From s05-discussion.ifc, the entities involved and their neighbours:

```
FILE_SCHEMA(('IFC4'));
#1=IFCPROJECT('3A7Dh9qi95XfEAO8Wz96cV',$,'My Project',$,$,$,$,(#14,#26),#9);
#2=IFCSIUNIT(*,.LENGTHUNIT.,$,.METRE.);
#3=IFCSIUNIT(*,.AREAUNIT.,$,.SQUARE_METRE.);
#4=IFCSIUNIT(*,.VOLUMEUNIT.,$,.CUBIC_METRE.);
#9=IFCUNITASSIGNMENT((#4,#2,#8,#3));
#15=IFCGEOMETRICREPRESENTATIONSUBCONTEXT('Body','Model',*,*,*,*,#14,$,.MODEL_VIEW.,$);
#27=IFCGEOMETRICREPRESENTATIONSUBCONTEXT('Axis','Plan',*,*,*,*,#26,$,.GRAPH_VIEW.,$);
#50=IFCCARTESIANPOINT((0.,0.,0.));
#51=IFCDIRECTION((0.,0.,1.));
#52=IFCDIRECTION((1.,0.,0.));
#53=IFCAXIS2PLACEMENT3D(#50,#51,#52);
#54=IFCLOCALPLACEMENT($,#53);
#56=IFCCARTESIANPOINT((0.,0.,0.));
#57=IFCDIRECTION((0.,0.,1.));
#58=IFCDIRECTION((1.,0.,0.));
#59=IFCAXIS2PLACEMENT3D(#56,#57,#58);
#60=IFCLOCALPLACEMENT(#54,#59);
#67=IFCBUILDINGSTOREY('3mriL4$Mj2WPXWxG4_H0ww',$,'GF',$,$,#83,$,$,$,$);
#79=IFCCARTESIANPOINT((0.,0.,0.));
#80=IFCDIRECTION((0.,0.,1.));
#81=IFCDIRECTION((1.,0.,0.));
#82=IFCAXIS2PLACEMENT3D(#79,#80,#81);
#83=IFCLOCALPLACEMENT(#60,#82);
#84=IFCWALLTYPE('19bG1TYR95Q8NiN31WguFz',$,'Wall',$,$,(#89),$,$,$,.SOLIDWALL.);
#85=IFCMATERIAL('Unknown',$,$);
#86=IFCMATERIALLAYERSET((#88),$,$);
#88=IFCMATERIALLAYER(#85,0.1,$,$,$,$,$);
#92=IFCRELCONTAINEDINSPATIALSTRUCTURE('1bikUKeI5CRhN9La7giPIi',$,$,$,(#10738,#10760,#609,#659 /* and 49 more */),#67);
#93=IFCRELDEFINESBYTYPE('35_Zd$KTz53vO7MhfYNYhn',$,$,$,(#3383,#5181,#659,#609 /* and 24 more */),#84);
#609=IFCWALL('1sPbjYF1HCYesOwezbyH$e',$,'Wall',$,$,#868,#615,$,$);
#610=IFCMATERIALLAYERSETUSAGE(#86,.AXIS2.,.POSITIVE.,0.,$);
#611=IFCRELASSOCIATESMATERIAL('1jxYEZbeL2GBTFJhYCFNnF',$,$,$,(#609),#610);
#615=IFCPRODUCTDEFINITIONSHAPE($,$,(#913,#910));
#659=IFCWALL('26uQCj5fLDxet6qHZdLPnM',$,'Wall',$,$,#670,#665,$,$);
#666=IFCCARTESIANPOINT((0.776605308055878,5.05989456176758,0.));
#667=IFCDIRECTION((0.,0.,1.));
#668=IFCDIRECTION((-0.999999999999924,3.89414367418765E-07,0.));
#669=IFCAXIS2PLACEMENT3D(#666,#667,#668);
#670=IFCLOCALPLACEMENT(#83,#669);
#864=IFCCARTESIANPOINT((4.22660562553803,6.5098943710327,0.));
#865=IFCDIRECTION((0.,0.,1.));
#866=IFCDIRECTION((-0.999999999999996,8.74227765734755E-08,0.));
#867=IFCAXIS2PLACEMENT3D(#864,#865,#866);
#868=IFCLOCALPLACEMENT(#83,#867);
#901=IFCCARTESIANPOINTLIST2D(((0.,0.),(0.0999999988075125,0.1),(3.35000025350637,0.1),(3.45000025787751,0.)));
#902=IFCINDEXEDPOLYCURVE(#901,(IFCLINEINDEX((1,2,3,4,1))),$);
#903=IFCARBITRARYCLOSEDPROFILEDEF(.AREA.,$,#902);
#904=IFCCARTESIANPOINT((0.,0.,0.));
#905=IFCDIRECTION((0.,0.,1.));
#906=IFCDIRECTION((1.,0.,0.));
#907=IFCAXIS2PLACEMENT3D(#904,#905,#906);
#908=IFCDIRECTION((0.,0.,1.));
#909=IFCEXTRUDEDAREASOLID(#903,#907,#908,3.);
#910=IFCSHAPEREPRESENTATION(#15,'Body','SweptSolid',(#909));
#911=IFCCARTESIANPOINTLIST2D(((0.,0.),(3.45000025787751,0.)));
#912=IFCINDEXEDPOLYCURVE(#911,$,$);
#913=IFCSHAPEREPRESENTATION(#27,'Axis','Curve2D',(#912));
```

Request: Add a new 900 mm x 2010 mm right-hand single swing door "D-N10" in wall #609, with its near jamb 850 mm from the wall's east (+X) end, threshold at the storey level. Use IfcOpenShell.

```python
import numpy as np
import ifcopenshell
import ifcopenshell.api.feature
import ifcopenshell.api.geometry
import ifcopenshell.api.root
import ifcopenshell.api.spatial
import ifcopenshell.geom
import ifcopenshell.util.element
import ifcopenshell.util.placement
import ifcopenshell.util.representation
import ifcopenshell.util.shape
import ifcopenshell.util.unit

model = ifcopenshell.open("s05-discussion.ifc")
unit_scale = ifcopenshell.util.unit.calculate_unit_scale(model)
settings = ifcopenshell.geom.settings()


def volume(element):
    """Net volume in cubic metres, openings subtracted."""
    shape = ifcopenshell.geom.create_shape(settings, element)
    return ifcopenshell.util.shape.get_volume(shape.geometry)


wall = model.by_id(609)
storey = ifcopenshell.util.element.get_container(wall, ifc_class="IfcBuildingStorey")
context = ifcopenshell.util.representation.get_context(model, "Model", "Body", "MODEL_VIEW")
before = volume(wall)

width, height, from_end, sill = 0.9, 2.01, 0.85, 0.0  # metres

# The wall runs along its own X axis, and the end named is its -X end.
wall_shape = ifcopenshell.geom.create_shape(settings, wall)
x, y, z = ifcopenshell.util.shape.get_vertices(wall_shape.geometry).T
start = x.min() + from_end
face, thickness = float(y.min()), float(y.max() - y.min())
wall_matrix = ifcopenshell.util.placement.get_local_placement(wall.ObjectPlacement)
level = ifcopenshell.util.placement.get_local_placement(storey.ObjectPlacement)[2, 3]


def in_wall(x, y):
    """Placement at x, y metres in the wall's axes, at sill height."""
    matrix = wall_matrix.copy()
    matrix[:, 3] = wall_matrix @ np.array([x / unit_scale, y / unit_scale, 0.0, 1.0])
    matrix[2, 3] = level + sill / unit_scale
    return matrix


# Opening: a box that overshoots both wall faces by 50 mm.
opening = ifcopenshell.api.root.create_entity(model, ifc_class="IfcOpeningElement", predefined_type="OPENING")
box = ifcopenshell.api.geometry.add_wall_representation(
    model, context=context, length=width, height=height, thickness=thickness + 0.1
)
ifcopenshell.api.geometry.assign_representation(model, product=opening, representation=box)
ifcopenshell.api.geometry.edit_object_placement(model, product=opening, matrix=in_wall(start, face - 0.05), is_si=False)
ifcopenshell.api.feature.add_feature(model, feature=opening, element=wall)

door = ifcopenshell.api.root.create_entity(model, ifc_class="IfcDoor", name="D-N10", predefined_type="DOOR")
door.OverallWidth, door.OverallHeight = width / unit_scale, height / unit_scale
door.OperationType = "SINGLE_SWING_RIGHT"
body = ifcopenshell.api.geometry.add_door_representation(
    model,
    context=context,
    overall_width=door.OverallWidth,
    overall_height=door.OverallHeight,
    operation_type="SINGLE_SWING_RIGHT",
    lining_properties={"LiningDepth": thickness / unit_scale, "ThresholdDepth": thickness / unit_scale},
)
ifcopenshell.api.geometry.assign_representation(model, product=door, representation=body)
ifcopenshell.api.spatial.assign_container(model, products=[door], relating_structure=storey)
ifcopenshell.api.feature.add_filling(model, opening=opening, element=door)

# The lining spans the wall, so the door starts at the wall face.
ifcopenshell.api.geometry.edit_object_placement(model, product=door, matrix=in_wall(start, face), is_si=False)

after = volume(wall)

print(f"wall volume {before:.3f} -> {after:.3f} m3")

model.write("s05-discussion_updated.ifc")
```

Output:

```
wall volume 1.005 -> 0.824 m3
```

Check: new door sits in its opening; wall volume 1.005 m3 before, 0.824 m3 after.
